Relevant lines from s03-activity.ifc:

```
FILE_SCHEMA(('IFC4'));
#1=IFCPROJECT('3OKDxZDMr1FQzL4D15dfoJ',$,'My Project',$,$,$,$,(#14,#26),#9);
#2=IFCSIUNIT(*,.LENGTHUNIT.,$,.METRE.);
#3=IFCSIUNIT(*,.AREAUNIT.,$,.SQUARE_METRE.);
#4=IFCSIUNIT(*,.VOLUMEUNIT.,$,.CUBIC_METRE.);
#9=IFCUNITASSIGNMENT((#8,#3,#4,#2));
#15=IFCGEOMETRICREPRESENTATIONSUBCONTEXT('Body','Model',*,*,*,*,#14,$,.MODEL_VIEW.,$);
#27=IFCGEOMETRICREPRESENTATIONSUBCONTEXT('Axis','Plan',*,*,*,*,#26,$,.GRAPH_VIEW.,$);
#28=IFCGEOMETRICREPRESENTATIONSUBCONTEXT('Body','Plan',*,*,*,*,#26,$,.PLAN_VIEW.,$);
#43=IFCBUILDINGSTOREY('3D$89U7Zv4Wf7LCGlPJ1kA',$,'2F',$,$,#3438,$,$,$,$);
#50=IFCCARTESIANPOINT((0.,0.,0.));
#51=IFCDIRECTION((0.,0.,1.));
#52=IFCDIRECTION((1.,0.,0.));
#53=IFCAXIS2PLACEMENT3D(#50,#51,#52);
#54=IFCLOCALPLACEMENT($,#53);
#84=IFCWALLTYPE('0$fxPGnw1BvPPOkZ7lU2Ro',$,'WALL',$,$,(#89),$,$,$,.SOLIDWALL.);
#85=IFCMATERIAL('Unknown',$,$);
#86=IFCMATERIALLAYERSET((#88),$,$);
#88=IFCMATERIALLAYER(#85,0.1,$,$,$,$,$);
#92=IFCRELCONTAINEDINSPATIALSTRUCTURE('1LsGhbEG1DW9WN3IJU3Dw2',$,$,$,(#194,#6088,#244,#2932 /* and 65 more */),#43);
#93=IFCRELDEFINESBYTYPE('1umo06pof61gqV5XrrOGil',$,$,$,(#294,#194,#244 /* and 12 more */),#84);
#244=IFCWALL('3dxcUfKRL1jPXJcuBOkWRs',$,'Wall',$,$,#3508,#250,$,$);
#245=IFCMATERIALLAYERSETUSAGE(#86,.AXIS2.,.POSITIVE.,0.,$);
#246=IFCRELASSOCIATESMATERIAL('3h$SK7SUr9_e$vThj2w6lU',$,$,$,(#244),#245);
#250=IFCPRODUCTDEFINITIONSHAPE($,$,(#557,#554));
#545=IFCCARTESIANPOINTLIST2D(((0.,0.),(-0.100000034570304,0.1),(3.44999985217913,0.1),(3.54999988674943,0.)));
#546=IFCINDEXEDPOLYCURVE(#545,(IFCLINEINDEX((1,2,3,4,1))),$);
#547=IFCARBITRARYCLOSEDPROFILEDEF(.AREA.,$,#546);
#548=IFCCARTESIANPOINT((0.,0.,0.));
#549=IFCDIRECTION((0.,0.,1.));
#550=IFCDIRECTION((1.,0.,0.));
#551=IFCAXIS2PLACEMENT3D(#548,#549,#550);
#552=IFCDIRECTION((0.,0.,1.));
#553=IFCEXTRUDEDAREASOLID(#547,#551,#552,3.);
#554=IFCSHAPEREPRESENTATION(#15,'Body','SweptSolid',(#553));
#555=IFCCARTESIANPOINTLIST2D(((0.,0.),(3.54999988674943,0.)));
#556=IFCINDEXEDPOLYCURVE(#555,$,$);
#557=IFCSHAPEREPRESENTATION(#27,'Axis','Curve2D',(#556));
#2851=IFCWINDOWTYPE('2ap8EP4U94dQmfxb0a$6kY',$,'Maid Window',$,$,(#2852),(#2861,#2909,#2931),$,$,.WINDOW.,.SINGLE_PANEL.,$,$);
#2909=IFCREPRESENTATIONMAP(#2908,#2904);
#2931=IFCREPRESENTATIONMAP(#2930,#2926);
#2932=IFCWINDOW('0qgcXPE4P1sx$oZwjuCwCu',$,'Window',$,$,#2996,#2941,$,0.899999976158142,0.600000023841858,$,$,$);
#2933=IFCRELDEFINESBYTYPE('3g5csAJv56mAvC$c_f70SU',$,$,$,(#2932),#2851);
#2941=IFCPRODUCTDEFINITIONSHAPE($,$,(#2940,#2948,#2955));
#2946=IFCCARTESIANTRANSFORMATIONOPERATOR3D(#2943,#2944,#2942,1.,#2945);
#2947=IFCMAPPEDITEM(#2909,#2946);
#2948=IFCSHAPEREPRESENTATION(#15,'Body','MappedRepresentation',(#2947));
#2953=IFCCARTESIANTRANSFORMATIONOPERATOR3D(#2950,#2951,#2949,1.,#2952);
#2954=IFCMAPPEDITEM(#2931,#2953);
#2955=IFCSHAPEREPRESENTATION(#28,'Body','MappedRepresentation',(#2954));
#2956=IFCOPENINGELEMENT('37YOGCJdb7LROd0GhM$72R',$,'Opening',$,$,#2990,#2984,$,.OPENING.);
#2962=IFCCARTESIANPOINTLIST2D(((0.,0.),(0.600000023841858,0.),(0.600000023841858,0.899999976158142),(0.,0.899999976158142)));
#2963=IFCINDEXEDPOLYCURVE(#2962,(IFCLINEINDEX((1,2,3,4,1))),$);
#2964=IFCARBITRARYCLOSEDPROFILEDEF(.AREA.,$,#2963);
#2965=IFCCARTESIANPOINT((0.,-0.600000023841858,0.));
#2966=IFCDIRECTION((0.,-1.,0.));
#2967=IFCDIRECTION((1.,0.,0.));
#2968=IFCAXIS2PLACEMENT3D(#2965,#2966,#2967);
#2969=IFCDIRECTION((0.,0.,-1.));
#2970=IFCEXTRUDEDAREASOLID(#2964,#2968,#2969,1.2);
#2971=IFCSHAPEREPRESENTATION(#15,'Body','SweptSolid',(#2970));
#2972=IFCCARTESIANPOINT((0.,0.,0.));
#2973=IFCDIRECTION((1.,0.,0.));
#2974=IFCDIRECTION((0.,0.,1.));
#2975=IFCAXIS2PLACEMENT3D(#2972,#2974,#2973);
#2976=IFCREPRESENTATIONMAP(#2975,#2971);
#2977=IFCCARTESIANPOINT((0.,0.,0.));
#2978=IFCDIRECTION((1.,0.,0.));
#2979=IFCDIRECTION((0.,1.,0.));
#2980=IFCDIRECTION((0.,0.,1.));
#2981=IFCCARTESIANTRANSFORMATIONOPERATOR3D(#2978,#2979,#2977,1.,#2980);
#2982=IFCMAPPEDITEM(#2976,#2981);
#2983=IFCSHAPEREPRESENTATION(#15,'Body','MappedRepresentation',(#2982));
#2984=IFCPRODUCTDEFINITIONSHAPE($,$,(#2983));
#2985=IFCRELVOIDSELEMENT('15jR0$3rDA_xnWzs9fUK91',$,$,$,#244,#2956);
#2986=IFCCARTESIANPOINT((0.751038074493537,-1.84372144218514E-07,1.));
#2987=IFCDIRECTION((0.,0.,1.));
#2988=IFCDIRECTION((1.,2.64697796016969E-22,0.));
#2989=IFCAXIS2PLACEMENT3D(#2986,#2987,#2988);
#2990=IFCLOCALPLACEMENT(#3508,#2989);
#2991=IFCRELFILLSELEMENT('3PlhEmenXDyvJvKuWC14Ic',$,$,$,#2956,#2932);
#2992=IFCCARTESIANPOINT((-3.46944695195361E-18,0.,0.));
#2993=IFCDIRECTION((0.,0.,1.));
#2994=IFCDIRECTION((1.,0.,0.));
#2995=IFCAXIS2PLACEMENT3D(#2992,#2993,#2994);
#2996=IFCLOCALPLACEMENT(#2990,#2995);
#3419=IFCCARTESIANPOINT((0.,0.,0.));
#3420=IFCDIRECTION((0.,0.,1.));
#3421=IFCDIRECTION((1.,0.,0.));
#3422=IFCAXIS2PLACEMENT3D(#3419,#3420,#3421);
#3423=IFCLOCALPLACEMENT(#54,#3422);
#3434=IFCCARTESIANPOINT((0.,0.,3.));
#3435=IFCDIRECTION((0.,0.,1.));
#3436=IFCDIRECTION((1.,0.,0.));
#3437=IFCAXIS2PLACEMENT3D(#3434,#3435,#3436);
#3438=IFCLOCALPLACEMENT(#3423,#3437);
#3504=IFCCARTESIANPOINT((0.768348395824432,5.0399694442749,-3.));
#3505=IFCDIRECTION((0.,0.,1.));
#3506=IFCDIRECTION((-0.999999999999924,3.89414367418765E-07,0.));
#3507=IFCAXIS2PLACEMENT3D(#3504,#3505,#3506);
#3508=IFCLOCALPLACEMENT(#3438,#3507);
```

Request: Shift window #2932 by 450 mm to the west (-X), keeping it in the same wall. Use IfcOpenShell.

```python
import ifcopenshell
import ifcopenshell.api.geometry
import ifcopenshell.util.placement
import ifcopenshell.util.unit

model = ifcopenshell.open("s03-activity.ifc")
unit_scale = ifcopenshell.util.unit.calculate_unit_scale(model)

window = model.by_id(2932)
opening = window.FillsVoids[0].RelatingOpeningElement
wall = opening.VoidsElements[0].RelatingBuildingElement

wall_matrix = ifcopenshell.util.placement.get_local_placement(wall.ObjectPlacement)
shift = wall_matrix[:3, 0] * 0.45 / unit_scale
before = ifcopenshell.util.placement.get_local_placement(window.ObjectPlacement)[:3, 3].copy()

# The window is placed relative to its opening, so it follows when the opening moves.
matrix = ifcopenshell.util.placement.get_local_placement(opening.ObjectPlacement)
matrix[:3, 3] += shift
ifcopenshell.api.geometry.edit_object_placement(
    model, product=opening, matrix=matrix, is_si=False, should_transform_children=True
)

after = ifcopenshell.util.placement.get_local_placement(window.ObjectPlacement)[:3, 3]
print("window moved by", (after - before).round(3) + 0.0)

model.write("s03-activity_v2.ifc")
```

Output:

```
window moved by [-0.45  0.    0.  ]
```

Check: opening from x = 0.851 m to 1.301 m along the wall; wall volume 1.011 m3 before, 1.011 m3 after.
